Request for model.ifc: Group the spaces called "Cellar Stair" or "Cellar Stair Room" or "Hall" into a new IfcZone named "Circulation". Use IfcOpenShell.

First a look at what the model holds.

```python
import ifcopenshell

model = ifcopenshell.open("model.ifc")
print(model.schema)
seen = {}
for space in model.by_type("IfcSpace"):
    seen[space.LongName] = seen.get(space.LongName, 0) + 1
for name, count in sorted(seen.items(), key=str):
    print(count, "x", name)
print("zones:", [z.Name for z in model.by_type("IfcZone")][:20])
```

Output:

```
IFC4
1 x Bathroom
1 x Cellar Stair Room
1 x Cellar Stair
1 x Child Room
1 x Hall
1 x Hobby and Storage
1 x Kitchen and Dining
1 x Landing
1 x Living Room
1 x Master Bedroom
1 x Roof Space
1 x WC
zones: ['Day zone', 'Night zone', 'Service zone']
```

```python
import ifcopenshell
import ifcopenshell.api.group
import ifcopenshell.api.root

model = ifcopenshell.open("model.ifc")

names = {"Cellar Stair", "Cellar Stair Room", "Hall"}
spaces = [s for s in model.by_type("IfcSpace") if s.LongName in names]

zone = ifcopenshell.api.root.create_entity(model, ifc_class="IfcZone", name="Circulation")
ifcopenshell.api.group.assign_group(model, products=spaces, group=zone)
print(len(spaces), "spaces in", zone.Name)

model.write("model-out.ifc")
```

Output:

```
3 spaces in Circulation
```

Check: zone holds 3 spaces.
